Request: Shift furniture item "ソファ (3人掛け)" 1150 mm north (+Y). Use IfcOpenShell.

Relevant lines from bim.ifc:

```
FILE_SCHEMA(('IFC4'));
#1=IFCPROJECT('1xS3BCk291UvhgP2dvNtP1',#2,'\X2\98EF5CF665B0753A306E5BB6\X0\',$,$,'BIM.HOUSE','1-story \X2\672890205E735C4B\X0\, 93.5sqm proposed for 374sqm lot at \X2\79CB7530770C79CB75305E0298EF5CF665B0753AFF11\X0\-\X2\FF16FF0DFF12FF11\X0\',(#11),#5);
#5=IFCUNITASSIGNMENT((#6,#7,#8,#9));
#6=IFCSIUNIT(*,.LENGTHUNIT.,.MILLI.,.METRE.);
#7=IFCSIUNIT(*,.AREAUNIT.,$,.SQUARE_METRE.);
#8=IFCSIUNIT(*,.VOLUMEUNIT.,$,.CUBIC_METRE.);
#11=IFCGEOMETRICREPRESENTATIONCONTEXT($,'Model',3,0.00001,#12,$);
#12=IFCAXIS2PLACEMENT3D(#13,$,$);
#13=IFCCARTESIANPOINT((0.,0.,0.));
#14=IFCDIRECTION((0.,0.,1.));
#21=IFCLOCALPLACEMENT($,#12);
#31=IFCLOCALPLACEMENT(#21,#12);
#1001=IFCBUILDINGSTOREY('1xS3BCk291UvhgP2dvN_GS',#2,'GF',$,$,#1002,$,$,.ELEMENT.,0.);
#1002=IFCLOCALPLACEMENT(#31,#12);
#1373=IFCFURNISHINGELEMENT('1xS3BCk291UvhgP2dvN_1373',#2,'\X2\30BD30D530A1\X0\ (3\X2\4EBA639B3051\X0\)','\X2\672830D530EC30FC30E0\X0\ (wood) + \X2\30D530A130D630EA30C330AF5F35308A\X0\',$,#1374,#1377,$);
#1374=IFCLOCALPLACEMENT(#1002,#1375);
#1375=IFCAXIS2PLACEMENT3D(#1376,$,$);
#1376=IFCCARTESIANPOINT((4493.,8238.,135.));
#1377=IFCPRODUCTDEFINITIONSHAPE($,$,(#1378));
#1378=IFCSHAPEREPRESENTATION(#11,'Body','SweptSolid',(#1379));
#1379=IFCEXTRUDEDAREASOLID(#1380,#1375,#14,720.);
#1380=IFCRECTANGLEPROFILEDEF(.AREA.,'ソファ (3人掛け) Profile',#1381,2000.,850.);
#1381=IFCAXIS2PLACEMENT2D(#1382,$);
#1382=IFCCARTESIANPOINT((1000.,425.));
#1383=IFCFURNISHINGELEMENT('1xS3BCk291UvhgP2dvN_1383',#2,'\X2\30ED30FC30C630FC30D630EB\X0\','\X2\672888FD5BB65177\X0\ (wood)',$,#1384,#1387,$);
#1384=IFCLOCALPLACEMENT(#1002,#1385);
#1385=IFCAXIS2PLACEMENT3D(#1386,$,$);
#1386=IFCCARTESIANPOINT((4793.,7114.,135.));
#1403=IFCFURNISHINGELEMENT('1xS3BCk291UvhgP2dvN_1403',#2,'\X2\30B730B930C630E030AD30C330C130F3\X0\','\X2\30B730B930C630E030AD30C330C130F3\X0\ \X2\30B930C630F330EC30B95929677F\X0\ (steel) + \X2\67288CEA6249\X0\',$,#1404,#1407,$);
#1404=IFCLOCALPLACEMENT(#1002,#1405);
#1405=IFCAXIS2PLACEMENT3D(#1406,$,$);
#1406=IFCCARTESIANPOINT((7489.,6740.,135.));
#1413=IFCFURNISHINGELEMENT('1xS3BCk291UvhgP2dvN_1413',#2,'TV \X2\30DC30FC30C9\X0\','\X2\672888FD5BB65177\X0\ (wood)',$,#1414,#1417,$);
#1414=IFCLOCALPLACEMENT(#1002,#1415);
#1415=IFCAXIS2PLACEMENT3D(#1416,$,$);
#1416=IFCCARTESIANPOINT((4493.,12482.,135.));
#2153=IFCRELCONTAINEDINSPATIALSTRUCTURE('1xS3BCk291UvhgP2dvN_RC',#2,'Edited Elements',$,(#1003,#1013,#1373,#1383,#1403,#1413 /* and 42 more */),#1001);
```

```python
import ifcopenshell
import ifcopenshell.api.geometry
import ifcopenshell.util.placement

model = ifcopenshell.open("bim.ifc")

item = model.by_guid("1xS3BCk291UvhgP2dvN_1373")
matrix = ifcopenshell.util.placement.get_local_placement(item.ObjectPlacement)
matrix[1, 3] += 1150.0
ifcopenshell.api.geometry.edit_object_placement(model, product=item, matrix=matrix, is_si=False)

print(ifcopenshell.util.placement.get_local_placement(item.ObjectPlacement).round(3) + 0.0)

model.write("bim_edited.ifc")
```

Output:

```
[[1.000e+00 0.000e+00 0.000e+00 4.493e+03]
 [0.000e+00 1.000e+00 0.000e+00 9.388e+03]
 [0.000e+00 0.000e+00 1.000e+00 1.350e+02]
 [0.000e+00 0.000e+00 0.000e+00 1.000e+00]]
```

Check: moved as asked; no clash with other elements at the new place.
